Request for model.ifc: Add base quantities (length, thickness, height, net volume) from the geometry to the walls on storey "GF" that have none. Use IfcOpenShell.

First a look at what the model holds.

```python
import ifcopenshell
import ifcopenshell.util.element
import ifcopenshell.util.unit

model = ifcopenshell.open("model.ifc")
print(model.schema)
for unit_type in ("LENGTHUNIT", "AREAUNIT", "VOLUMEUNIT"):
    print(unit_type, ifcopenshell.util.unit.calculate_unit_scale(model, unit_type))
storey = next(s for s in model.by_type("IfcBuildingStorey") if s.Name == "GF")
walls = [e for e in ifcopenshell.util.element.get_decomposition(storey) if e.is_a("IfcWall")]
for e in sorted(walls, key=lambda e: e.id()):
    print(e.id(), e.is_a(), e.Name, list(ifcopenshell.util.element.get_psets(e, qtos_only=True)), sep=" | ")
```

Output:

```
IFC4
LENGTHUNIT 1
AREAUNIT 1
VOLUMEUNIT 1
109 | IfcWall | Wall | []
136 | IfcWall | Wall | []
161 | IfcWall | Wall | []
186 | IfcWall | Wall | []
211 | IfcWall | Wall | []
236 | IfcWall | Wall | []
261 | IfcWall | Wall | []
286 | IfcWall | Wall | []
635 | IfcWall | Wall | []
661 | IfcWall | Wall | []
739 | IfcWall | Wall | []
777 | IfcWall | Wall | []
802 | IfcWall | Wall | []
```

```python
import ifcopenshell
import ifcopenshell.api.pset
import ifcopenshell.geom
import ifcopenshell.util.element
import ifcopenshell.util.shape
import ifcopenshell.util.unit

model = ifcopenshell.open("model.ifc")
unit_scale = ifcopenshell.util.unit.calculate_unit_scale(model)
volume_scale = ifcopenshell.util.unit.calculate_unit_scale(model, "VOLUMEUNIT")
settings = ifcopenshell.geom.settings()

storey = next(s for s in model.by_type("IfcBuildingStorey") if s.Name == "GF")
walls = [e for e in ifcopenshell.util.element.get_decomposition(storey) if e.is_a("IfcWall")]

for e in sorted(walls, key=lambda e: e.id()):
    if ifcopenshell.util.element.get_psets(e, qtos_only=True, should_inherit=False):
        continue
    # Geometry comes back in metres, in the element's own axes.
    shape = ifcopenshell.geom.create_shape(settings, e)
    values = {
        "Length": ifcopenshell.util.shape.get_x(shape.geometry) / unit_scale,
        "Width": ifcopenshell.util.shape.get_y(shape.geometry) / unit_scale,
        "Height": ifcopenshell.util.shape.get_z(shape.geometry) / unit_scale,
        "NetVolume": ifcopenshell.util.shape.get_volume(shape.geometry) / volume_scale,
    }
    qto = ifcopenshell.api.pset.add_qto(model, product=e, name="Qto_WallBaseQuantities")
    ifcopenshell.api.pset.edit_qto(model, qto=qto, properties=values)
    print(e.id(), {k: round(v, 3) for k, v in values.items()})

model.write("model_edited.ifc")
```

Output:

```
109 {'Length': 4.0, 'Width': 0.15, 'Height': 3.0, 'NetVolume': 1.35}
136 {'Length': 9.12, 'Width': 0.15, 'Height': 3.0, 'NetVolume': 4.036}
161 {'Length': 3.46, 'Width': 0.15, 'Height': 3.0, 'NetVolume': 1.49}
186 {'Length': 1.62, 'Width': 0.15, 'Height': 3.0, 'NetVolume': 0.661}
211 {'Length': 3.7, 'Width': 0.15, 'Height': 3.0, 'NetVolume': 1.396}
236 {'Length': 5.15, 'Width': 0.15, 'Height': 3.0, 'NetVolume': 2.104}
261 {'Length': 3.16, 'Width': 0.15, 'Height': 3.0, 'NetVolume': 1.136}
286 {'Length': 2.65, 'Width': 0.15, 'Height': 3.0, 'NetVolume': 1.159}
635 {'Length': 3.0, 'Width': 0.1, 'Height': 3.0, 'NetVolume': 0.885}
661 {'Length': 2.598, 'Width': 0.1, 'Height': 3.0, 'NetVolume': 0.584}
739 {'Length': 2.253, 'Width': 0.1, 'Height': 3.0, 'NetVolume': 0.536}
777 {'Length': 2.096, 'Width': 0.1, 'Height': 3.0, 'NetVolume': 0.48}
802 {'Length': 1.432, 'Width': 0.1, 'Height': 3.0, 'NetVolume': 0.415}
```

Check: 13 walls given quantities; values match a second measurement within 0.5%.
